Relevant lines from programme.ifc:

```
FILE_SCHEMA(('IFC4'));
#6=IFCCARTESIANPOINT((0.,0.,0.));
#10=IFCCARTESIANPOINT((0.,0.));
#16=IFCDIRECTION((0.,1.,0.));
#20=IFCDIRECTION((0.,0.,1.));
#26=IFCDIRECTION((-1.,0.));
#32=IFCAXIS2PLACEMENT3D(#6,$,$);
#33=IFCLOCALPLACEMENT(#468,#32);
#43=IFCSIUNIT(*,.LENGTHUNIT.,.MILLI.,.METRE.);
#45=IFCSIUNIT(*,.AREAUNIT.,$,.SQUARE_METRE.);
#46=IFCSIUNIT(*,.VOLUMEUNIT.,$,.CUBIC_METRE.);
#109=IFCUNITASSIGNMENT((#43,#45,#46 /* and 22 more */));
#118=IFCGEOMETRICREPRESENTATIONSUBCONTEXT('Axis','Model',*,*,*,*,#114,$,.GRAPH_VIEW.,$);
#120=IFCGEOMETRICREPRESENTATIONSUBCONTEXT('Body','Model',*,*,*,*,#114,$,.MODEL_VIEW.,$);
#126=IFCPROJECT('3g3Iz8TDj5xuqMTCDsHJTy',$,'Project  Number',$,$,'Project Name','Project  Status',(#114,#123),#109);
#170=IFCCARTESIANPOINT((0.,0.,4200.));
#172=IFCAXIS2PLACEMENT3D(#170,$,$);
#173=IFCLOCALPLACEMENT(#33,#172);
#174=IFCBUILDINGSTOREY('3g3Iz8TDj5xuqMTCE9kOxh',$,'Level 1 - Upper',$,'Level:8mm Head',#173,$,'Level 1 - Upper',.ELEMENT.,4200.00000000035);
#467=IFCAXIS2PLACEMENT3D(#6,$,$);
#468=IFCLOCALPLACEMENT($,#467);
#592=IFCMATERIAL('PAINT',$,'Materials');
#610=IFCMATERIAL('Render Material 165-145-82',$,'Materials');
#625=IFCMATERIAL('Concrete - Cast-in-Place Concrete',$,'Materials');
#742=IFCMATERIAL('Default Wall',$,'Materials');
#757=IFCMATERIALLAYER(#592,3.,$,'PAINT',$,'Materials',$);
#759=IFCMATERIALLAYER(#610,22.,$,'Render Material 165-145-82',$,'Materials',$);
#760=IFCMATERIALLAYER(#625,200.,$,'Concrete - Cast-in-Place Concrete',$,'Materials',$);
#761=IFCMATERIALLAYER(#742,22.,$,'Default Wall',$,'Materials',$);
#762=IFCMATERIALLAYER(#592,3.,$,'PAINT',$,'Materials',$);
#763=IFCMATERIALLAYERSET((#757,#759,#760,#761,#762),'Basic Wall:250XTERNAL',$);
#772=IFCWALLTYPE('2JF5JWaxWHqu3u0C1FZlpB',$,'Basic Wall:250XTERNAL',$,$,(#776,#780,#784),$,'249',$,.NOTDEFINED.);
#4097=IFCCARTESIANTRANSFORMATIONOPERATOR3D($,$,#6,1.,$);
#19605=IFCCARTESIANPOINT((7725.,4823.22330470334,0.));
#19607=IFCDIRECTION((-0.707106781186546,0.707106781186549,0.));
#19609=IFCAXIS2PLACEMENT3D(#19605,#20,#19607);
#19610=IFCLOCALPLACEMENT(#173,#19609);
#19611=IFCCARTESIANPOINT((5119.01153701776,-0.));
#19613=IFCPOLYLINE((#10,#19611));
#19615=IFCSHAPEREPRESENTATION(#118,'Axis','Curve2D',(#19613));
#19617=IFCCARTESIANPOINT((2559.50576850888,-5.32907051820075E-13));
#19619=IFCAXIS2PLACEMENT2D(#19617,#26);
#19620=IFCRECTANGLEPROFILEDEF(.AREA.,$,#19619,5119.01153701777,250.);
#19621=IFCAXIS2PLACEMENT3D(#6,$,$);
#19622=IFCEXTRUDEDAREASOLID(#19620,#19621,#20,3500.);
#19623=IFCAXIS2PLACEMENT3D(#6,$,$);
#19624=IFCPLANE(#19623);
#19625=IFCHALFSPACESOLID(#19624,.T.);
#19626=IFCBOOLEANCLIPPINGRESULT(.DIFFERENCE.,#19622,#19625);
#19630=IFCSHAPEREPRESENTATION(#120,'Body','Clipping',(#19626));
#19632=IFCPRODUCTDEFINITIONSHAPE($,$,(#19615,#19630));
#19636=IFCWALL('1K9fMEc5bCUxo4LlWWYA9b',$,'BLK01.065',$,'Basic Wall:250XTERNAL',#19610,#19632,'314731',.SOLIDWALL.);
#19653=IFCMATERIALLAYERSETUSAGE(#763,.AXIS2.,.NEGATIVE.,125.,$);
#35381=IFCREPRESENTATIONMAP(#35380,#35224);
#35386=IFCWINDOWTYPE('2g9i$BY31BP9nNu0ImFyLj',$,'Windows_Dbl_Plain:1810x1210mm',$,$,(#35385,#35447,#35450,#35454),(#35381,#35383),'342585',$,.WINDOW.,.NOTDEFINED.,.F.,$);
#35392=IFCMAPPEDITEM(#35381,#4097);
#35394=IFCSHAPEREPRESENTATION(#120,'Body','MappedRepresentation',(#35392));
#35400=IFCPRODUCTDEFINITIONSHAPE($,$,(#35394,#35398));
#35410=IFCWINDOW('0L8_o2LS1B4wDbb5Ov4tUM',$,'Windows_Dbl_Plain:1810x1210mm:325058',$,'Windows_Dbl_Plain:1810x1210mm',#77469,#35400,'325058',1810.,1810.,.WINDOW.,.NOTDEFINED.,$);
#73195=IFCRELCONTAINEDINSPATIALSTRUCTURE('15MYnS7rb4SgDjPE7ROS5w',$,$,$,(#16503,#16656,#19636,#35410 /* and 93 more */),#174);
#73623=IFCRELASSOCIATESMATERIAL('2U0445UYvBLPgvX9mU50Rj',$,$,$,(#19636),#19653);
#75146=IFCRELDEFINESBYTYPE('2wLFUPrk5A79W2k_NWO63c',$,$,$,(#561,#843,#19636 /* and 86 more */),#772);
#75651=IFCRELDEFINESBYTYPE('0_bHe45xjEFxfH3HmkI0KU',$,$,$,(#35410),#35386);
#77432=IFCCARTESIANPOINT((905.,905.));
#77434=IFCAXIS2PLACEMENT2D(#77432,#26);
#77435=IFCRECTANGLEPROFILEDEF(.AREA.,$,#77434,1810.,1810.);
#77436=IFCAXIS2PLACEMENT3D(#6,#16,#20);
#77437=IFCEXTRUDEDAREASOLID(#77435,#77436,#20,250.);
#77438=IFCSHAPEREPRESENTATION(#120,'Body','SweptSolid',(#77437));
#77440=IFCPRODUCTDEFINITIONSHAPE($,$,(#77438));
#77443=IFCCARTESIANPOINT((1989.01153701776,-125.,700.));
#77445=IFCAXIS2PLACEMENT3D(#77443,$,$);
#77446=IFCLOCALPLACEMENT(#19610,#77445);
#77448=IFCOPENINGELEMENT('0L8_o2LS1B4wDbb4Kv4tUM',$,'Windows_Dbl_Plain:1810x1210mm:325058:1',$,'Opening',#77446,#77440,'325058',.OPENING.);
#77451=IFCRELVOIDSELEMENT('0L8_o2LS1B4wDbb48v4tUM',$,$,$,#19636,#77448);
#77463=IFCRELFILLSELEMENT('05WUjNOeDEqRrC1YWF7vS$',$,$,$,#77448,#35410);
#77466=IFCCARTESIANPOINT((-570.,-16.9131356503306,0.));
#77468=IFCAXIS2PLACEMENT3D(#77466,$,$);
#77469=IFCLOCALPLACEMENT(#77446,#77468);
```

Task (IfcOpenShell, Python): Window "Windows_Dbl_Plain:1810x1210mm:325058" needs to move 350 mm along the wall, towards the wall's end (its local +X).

```python
import ifcopenshell
import ifcopenshell.api.geometry
import ifcopenshell.util.placement
import ifcopenshell.util.unit

model = ifcopenshell.open("programme.ifc")
unit_scale = ifcopenshell.util.unit.calculate_unit_scale(model)

window = model.by_guid("0L8_o2LS1B4wDbb5Ov4tUM")
opening = window.FillsVoids[0].RelatingOpeningElement
wall = opening.VoidsElements[0].RelatingBuildingElement

wall_matrix = ifcopenshell.util.placement.get_local_placement(wall.ObjectPlacement)
shift = wall_matrix[:3, 0] * 0.35 / unit_scale
before = ifcopenshell.util.placement.get_local_placement(window.ObjectPlacement)[:3, 3].copy()

# The window is placed relative to its opening, so it follows when the opening moves.
matrix = ifcopenshell.util.placement.get_local_placement(opening.ObjectPlacement)
matrix[:3, 3] += shift
ifcopenshell.api.geometry.edit_object_placement(
    model, product=opening, matrix=matrix, is_si=False, should_transform_children=True
)

after = ifcopenshell.util.placement.get_local_placement(window.ObjectPlacement)[:3, 3]
print("window moved by", (after - before).round(3) + 0.0)

model.write("programme_v2.ifc")
```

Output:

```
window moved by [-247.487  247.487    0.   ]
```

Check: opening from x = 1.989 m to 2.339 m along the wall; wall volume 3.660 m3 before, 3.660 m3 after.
